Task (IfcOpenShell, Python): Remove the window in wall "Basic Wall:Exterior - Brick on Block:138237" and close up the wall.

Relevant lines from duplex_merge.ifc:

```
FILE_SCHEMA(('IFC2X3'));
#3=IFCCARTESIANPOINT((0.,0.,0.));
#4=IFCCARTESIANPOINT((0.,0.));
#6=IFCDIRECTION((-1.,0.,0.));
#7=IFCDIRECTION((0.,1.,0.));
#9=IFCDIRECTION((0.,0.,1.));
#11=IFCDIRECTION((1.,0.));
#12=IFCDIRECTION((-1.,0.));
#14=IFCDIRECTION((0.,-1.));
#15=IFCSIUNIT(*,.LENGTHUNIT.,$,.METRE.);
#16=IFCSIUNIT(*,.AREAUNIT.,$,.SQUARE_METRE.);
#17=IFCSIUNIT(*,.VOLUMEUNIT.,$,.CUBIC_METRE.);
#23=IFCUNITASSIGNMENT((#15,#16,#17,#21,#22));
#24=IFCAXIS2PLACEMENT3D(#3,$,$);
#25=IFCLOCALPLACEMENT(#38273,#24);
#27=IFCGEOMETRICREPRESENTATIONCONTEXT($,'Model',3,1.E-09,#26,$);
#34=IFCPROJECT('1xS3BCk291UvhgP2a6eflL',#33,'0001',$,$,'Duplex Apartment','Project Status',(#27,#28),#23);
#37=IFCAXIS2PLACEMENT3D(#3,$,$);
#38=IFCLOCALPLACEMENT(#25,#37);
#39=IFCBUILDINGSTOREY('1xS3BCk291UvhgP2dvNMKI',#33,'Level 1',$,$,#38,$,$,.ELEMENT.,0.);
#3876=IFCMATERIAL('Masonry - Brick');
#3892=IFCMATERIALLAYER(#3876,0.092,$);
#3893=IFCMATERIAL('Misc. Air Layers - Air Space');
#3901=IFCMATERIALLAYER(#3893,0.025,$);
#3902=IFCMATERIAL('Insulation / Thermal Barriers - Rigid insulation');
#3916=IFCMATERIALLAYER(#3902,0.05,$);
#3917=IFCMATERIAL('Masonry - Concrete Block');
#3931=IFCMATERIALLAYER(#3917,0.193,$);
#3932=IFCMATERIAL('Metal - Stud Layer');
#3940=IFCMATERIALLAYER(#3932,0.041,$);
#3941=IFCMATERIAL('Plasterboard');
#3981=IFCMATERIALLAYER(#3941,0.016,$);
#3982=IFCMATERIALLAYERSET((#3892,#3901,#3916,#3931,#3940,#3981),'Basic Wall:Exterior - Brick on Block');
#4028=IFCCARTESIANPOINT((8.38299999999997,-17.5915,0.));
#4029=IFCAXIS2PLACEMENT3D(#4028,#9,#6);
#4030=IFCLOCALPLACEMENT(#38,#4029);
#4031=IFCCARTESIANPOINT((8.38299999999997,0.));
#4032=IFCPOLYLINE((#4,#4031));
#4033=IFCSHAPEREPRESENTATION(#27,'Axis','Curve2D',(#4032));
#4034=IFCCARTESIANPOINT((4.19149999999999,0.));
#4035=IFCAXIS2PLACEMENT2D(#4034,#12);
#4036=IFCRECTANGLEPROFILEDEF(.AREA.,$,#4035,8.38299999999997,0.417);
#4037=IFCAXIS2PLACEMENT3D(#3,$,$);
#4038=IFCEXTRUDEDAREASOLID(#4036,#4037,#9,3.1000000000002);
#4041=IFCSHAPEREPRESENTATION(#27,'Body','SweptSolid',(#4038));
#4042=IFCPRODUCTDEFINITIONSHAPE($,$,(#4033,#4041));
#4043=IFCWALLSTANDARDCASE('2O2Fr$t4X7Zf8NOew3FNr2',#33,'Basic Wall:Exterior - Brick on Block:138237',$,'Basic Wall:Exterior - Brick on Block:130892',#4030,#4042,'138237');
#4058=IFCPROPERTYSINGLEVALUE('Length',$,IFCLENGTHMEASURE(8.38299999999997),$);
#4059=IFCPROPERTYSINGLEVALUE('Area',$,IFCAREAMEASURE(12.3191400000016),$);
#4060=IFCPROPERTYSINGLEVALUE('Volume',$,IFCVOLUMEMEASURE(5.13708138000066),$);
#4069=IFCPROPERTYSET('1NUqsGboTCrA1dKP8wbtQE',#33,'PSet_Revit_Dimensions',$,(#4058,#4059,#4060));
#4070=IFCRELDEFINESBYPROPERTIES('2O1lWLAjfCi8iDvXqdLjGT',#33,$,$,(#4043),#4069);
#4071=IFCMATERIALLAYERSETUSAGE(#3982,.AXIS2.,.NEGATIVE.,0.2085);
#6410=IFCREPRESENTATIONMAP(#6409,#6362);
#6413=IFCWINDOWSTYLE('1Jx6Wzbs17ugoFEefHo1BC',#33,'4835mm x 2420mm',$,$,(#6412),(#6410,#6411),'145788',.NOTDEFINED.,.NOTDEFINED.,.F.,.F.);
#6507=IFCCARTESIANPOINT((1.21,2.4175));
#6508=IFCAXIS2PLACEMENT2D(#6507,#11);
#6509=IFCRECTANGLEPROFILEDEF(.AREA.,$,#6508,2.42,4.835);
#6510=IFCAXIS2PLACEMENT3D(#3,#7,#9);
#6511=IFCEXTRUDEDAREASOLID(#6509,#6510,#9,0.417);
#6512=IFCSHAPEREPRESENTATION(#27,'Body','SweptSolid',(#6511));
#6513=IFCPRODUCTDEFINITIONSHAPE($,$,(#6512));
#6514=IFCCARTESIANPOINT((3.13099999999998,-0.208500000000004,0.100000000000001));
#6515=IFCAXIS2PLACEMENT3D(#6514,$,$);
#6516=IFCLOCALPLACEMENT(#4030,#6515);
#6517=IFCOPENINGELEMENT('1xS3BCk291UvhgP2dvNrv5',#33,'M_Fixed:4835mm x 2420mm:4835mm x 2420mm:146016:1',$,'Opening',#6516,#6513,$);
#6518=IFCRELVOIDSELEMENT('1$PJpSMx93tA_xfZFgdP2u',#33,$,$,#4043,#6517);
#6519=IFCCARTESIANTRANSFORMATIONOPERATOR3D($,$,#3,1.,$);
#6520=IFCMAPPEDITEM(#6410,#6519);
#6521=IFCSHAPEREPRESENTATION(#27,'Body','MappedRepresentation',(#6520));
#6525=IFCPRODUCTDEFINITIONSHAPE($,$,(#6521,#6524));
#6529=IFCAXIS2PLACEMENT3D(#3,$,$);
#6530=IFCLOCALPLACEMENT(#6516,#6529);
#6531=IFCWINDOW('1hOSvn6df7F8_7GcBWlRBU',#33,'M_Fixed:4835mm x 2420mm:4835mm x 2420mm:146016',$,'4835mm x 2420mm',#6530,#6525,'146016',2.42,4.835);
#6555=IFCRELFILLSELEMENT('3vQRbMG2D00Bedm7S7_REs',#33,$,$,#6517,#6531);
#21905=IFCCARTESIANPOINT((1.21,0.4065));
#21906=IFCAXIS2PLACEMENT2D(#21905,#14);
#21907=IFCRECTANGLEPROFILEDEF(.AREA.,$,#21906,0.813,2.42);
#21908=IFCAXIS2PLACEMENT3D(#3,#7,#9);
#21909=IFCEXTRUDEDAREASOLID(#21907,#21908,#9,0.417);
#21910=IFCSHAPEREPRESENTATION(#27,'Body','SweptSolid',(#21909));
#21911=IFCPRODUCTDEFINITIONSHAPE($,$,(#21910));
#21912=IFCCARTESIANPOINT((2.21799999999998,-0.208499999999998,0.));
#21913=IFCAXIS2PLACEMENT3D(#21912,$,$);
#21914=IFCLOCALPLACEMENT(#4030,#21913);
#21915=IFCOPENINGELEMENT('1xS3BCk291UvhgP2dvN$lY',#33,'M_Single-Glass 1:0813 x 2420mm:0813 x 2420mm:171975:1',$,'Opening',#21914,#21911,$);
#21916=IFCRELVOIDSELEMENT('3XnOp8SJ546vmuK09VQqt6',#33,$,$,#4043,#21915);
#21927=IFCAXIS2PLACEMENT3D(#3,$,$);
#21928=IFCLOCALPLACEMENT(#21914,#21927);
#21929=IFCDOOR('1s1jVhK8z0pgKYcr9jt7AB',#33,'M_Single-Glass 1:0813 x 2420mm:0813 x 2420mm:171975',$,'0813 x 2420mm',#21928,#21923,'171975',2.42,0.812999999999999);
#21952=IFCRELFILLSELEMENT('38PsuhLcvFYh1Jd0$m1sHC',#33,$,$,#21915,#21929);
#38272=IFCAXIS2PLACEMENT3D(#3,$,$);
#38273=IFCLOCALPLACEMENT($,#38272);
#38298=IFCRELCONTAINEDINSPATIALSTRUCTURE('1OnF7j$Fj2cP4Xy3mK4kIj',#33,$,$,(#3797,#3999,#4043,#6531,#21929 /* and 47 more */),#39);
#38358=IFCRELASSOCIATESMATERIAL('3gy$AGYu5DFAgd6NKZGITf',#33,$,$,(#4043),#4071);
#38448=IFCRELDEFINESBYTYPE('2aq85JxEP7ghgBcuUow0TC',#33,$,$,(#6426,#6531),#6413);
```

```python
import ifcopenshell
import ifcopenshell.api.feature
import ifcopenshell.api.pset
import ifcopenshell.api.root
import ifcopenshell.geom
import ifcopenshell.util.element
import ifcopenshell.util.shape
import ifcopenshell.util.unit

model = ifcopenshell.open("duplex_merge.ifc")
area_scale = ifcopenshell.util.unit.calculate_unit_scale(model, "AREAUNIT")
volume_scale = ifcopenshell.util.unit.calculate_unit_scale(model, "VOLUMEUNIT")
settings = ifcopenshell.geom.settings()


def volume(element):
    """Net volume in cubic metres, openings subtracted."""
    shape = ifcopenshell.geom.create_shape(settings, element)
    return ifcopenshell.util.shape.get_volume(shape.geometry)


window = model.by_guid("1hOSvn6df7F8_7GcBWlRBU")
opening = window.FillsVoids[0].RelatingOpeningElement
wall = opening.VoidsElements[0].RelatingBuildingElement
before = volume(wall)

ifcopenshell.api.root.remove_product(model, product=window)
ifcopenshell.api.feature.remove_feature(model, feature=opening)

after = volume(wall)
thickness = 0.417  # wall thickness in metres

# Update the wall's stored quantities.
pset = model.by_id(ifcopenshell.util.element.get_pset(wall, "PSet_Revit_Dimensions", should_inherit=False)["id"])
ifcopenshell.api.pset.edit_pset(model, pset=pset, properties={
    "Area": model.create_entity("IfcAreaMeasure", after / thickness / area_scale),
    "Volume": model.create_entity("IfcVolumeMeasure", after / volume_scale),
})

print(f"wall volume {before:.3f} -> {after:.3f} m3")

model.write("duplex_merge_v2.ifc")
```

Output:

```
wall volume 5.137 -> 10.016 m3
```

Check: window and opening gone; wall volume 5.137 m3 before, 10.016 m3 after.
